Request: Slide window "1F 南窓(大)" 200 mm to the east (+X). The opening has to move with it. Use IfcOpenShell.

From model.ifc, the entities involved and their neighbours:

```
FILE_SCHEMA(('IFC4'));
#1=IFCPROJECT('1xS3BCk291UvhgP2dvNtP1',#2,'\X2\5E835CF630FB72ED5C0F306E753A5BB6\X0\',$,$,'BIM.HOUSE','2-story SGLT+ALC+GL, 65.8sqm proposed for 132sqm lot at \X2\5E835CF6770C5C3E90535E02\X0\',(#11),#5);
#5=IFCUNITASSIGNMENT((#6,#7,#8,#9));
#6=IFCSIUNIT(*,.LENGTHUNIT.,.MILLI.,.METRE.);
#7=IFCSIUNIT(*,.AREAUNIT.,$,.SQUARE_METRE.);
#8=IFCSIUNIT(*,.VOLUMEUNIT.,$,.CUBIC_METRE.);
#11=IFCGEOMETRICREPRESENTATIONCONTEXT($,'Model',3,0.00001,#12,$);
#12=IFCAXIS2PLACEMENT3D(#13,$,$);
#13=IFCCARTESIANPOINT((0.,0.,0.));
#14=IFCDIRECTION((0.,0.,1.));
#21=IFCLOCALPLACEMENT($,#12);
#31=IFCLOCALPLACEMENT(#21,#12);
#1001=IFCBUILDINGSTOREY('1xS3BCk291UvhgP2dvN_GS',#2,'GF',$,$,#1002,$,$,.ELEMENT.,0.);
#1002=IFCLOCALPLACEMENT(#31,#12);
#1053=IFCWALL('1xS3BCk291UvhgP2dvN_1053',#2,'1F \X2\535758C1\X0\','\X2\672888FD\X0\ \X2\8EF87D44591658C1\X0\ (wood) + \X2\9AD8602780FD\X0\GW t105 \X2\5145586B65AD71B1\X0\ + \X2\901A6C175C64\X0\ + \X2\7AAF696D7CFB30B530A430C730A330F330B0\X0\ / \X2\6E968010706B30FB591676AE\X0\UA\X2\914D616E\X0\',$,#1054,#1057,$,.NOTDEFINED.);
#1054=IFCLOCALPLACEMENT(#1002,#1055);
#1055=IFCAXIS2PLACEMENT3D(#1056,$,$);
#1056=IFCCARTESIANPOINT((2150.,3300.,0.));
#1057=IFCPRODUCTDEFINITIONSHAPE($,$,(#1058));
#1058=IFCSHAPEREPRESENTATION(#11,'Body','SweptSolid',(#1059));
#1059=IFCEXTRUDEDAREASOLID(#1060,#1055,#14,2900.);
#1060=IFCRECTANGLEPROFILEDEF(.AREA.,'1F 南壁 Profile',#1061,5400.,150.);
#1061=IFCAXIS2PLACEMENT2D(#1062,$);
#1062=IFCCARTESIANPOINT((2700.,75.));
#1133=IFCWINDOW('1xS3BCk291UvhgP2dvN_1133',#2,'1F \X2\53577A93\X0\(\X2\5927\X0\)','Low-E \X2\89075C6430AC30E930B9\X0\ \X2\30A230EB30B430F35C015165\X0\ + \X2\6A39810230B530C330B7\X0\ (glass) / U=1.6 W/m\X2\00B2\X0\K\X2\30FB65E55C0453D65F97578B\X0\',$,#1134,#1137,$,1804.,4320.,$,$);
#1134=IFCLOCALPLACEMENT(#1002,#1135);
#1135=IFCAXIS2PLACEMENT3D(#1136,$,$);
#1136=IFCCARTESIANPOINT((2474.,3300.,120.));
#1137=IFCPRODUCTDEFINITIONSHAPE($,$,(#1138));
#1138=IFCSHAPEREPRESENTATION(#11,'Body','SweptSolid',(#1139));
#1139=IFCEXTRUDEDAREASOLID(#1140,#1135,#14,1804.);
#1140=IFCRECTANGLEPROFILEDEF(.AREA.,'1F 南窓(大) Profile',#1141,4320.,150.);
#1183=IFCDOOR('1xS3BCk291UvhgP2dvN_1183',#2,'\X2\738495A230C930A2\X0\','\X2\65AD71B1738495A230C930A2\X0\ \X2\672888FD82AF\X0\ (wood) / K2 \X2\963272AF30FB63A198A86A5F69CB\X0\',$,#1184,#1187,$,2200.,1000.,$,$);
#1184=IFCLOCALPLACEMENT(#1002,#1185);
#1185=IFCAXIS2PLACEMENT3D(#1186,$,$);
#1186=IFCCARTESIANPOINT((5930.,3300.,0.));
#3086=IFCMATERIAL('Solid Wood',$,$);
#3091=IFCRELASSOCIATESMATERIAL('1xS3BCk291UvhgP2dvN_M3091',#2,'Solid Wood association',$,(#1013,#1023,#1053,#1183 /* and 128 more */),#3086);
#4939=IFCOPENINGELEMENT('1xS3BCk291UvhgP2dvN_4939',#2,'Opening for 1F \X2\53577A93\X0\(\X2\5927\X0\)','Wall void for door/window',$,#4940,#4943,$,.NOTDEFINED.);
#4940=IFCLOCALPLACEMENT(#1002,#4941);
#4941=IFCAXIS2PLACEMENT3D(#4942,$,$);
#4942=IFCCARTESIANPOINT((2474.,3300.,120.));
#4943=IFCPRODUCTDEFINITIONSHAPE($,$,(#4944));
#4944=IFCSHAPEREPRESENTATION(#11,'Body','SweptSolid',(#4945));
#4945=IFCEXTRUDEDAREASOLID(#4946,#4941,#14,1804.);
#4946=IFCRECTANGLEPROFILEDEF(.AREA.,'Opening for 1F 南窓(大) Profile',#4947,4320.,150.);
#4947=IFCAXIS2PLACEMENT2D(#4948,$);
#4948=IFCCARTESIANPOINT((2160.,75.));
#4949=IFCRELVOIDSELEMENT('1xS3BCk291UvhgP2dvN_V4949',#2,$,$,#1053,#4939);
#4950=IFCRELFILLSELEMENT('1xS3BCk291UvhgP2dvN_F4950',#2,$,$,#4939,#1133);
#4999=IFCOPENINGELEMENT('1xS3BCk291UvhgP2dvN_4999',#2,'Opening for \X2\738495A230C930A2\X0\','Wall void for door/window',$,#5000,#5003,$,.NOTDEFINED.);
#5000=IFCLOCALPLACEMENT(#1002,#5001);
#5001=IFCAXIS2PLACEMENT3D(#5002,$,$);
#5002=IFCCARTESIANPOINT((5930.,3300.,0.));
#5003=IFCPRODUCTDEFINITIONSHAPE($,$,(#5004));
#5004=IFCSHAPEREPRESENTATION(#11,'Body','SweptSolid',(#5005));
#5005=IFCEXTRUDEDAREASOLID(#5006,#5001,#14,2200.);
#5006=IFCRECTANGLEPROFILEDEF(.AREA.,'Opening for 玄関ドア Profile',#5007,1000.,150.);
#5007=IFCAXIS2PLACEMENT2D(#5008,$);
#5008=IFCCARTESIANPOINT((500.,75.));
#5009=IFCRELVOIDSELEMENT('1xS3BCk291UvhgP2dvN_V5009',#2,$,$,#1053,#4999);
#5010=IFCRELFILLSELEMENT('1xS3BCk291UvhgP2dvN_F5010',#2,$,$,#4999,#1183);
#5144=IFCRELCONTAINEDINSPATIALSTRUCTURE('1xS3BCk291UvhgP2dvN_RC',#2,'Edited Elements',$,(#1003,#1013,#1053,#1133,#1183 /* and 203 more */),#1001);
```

```python
import ifcopenshell
import ifcopenshell.api.geometry
import ifcopenshell.util.placement
import ifcopenshell.util.unit

model = ifcopenshell.open("model.ifc")
unit_scale = ifcopenshell.util.unit.calculate_unit_scale(model)

window = model.by_guid("1xS3BCk291UvhgP2dvN_1133")
opening = window.FillsVoids[0].RelatingOpeningElement
wall = opening.VoidsElements[0].RelatingBuildingElement

wall_matrix = ifcopenshell.util.placement.get_local_placement(wall.ObjectPlacement)
shift = wall_matrix[:3, 0] * 0.2 / unit_scale
before = ifcopenshell.util.placement.get_local_placement(window.ObjectPlacement)[:3, 3].copy()

# The window is not placed relative to its opening, so move both.
for product in (opening, window):
    matrix = ifcopenshell.util.placement.get_local_placement(product.ObjectPlacement)
    matrix[:3, 3] += shift
    ifcopenshell.api.geometry.edit_object_placement(model, product=product, matrix=matrix, is_si=False)

after = ifcopenshell.util.placement.get_local_placement(window.ObjectPlacement)[:3, 3]
print("window moved by", (after - before).round(3) + 0.0)

model.write("model_v2.ifc")
```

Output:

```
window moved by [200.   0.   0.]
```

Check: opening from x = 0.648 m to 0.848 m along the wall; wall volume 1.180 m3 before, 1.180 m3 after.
